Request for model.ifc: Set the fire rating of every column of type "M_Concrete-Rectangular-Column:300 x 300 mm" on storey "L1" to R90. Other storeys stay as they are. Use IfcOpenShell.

First a look at what the model holds.

```python
import ifcopenshell
import ifcopenshell.util.element

model = ifcopenshell.open("model.ifc")
print(model.schema)
storey = next(s for s in model.by_type("IfcBuildingStorey") if s.Name == "L1")
columns = [e for e in ifcopenshell.util.element.get_decomposition(storey) if e.is_a("IfcColumn")]
seen = {}
for e in columns:
    element_type = ifcopenshell.util.element.get_type(e)
    key = (element_type.Name if element_type != e and element_type else None, ifcopenshell.util.element.get_pset(e, "Pset_ColumnCommon", "FireRating"))
    seen[key] = seen.get(key, 0) + 1
for (name, value), count in sorted(seen.items(), key=str):
    print(count, "x", name, "|", value)
```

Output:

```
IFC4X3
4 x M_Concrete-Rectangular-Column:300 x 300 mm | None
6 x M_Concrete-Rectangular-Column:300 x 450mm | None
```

```python
import ifcopenshell
import ifcopenshell.api.pset
import ifcopenshell.util.element

model = ifcopenshell.open("model.ifc")

storey = next(s for s in model.by_type("IfcBuildingStorey") if s.Name == "L1")
columns = [e for e in ifcopenshell.util.element.get_decomposition(storey) if e.is_a("IfcColumn")]

count = 0
for e in columns:
    element_type = ifcopenshell.util.element.get_type(e)
    if element_type in (None, e) or element_type.Name != "M_Concrete-Rectangular-Column:300 x 300 mm":
        continue
    # add_pset returns the element's existing set when there is one.
    pset = ifcopenshell.api.pset.add_pset(model, product=e, name="Pset_ColumnCommon")
    ifcopenshell.api.pset.edit_pset(model, pset=pset, properties={"FireRating": "R90"})
    count += 1

print(count, "columns updated")

model.write("model_v2.ifc")
```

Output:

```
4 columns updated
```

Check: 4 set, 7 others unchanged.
